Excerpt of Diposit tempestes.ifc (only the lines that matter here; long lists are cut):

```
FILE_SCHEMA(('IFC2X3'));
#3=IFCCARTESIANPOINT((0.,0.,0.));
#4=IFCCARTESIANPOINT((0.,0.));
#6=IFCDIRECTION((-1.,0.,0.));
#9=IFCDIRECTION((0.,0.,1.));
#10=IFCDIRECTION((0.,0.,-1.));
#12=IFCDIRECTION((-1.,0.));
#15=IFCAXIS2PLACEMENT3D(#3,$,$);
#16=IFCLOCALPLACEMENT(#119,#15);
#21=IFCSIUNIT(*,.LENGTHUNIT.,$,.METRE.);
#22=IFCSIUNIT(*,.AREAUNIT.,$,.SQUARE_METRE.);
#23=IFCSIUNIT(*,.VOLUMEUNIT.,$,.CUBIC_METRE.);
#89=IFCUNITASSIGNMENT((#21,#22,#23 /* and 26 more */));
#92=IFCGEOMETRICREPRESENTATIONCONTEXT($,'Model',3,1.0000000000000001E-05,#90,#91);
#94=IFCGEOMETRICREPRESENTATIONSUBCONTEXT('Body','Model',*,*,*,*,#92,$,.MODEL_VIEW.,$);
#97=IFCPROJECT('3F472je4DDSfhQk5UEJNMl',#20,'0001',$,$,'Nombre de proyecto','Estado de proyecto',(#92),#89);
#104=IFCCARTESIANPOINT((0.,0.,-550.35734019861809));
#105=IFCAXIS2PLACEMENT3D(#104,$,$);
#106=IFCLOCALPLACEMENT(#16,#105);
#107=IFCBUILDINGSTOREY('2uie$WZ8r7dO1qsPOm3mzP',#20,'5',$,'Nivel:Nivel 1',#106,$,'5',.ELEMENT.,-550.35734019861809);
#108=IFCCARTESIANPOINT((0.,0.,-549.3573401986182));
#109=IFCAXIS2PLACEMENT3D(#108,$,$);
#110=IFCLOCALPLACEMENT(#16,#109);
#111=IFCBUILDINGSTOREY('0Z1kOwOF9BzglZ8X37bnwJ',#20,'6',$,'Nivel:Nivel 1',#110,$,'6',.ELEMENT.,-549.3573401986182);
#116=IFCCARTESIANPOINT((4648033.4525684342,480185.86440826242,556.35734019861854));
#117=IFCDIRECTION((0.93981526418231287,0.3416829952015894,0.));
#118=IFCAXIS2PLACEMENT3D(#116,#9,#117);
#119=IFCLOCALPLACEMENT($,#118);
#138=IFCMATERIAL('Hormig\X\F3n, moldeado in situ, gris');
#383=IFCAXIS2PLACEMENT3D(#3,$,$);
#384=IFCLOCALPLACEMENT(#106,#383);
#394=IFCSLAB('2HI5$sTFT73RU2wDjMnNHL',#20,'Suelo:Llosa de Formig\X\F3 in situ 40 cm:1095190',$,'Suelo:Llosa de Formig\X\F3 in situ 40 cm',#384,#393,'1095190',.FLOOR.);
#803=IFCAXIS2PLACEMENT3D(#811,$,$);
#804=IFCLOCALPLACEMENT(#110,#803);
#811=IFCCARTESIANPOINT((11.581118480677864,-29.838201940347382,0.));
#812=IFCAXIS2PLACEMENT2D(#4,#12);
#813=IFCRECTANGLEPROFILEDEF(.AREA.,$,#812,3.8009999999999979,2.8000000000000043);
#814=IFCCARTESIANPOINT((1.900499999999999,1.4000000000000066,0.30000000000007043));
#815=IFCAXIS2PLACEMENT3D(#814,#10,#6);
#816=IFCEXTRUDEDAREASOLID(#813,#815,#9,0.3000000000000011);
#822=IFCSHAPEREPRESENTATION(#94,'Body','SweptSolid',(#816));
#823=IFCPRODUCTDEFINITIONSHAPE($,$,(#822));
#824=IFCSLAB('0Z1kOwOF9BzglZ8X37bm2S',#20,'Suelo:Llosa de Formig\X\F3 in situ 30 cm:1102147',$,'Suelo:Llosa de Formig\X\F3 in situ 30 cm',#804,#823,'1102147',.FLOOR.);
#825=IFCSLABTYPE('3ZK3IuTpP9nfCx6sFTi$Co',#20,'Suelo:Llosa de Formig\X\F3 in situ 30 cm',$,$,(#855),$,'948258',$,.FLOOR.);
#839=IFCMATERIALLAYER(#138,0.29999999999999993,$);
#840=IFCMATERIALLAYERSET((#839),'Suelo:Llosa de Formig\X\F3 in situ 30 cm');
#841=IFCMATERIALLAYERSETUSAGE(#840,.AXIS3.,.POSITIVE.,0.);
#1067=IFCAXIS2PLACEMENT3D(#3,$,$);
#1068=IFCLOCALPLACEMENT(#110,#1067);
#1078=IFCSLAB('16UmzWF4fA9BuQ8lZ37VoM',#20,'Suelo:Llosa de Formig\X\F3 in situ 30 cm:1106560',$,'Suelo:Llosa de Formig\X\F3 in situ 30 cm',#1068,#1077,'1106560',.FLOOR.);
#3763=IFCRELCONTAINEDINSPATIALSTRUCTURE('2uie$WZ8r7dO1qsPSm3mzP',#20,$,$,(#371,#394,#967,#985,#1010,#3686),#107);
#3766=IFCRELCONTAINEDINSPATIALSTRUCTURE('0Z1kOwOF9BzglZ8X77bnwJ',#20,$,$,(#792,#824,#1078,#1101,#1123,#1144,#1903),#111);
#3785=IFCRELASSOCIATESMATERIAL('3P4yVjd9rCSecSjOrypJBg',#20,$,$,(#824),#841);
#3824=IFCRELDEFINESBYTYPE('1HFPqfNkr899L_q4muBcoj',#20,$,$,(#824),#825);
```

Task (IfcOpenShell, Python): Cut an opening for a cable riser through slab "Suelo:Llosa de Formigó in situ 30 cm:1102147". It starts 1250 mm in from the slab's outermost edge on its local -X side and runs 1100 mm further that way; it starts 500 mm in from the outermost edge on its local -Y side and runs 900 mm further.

```python
import numpy as np
import ifcopenshell
import ifcopenshell.api.feature
import ifcopenshell.api.geometry
import ifcopenshell.api.root
import ifcopenshell.geom
import ifcopenshell.util.placement
import ifcopenshell.util.representation
import ifcopenshell.util.shape
import ifcopenshell.util.unit

model = ifcopenshell.open("Diposit tempestes.ifc")
unit_scale = ifcopenshell.util.unit.calculate_unit_scale(model)
settings = ifcopenshell.geom.settings()


def volume(element):
    """Net volume in cubic metres, openings subtracted."""
    shape = ifcopenshell.geom.create_shape(settings, element)
    return ifcopenshell.util.shape.get_volume(shape.geometry)


slab = model.by_id(824)
before = volume(slab)

# Extent in the slab's own axes, in metres. The edges named are its -X and -Y sides.
slab_shape = ifcopenshell.geom.create_shape(settings, slab)
vertices = ifcopenshell.util.shape.get_vertices(slab_shape.geometry)
x_min, y_min, bottom = vertices.min(axis=0)
top = vertices[:, 2].max()

opening = ifcopenshell.api.root.create_entity(model, ifc_class="IfcOpeningElement", name="Cable riser opening")
context = ifcopenshell.util.representation.get_context(model, "Model", "Body", "MODEL_VIEW")
width, depth = 1.1, 0.9
outline = [(0.0, 0.0), (width, 0.0), (width, depth), (0.0, depth), (0.0, 0.0)]
# Overshoot both faces by 50 mm so the cut is clean.
shape = ifcopenshell.api.geometry.add_slab_representation(
    model, context=context, depth=top - bottom + 0.1, polyline=outline
)
ifcopenshell.api.geometry.assign_representation(model, product=opening, representation=shape)

matrix = ifcopenshell.util.placement.get_local_placement(slab.ObjectPlacement)
matrix[:, 3] = matrix @ np.append(np.array([x_min + 1.25, y_min + 0.5, bottom - 0.05]) / unit_scale, 1.0)
ifcopenshell.api.geometry.edit_object_placement(model, product=opening, matrix=matrix, is_si=False)
ifcopenshell.api.feature.add_feature(model, feature=opening, element=slab)

after = volume(slab)

print(f"slab volume {before:.3f} -> {after:.3f} m3")

model.write("Diposit tempestes_v2.ifc")
```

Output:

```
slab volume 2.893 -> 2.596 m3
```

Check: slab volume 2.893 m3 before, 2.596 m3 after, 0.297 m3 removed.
